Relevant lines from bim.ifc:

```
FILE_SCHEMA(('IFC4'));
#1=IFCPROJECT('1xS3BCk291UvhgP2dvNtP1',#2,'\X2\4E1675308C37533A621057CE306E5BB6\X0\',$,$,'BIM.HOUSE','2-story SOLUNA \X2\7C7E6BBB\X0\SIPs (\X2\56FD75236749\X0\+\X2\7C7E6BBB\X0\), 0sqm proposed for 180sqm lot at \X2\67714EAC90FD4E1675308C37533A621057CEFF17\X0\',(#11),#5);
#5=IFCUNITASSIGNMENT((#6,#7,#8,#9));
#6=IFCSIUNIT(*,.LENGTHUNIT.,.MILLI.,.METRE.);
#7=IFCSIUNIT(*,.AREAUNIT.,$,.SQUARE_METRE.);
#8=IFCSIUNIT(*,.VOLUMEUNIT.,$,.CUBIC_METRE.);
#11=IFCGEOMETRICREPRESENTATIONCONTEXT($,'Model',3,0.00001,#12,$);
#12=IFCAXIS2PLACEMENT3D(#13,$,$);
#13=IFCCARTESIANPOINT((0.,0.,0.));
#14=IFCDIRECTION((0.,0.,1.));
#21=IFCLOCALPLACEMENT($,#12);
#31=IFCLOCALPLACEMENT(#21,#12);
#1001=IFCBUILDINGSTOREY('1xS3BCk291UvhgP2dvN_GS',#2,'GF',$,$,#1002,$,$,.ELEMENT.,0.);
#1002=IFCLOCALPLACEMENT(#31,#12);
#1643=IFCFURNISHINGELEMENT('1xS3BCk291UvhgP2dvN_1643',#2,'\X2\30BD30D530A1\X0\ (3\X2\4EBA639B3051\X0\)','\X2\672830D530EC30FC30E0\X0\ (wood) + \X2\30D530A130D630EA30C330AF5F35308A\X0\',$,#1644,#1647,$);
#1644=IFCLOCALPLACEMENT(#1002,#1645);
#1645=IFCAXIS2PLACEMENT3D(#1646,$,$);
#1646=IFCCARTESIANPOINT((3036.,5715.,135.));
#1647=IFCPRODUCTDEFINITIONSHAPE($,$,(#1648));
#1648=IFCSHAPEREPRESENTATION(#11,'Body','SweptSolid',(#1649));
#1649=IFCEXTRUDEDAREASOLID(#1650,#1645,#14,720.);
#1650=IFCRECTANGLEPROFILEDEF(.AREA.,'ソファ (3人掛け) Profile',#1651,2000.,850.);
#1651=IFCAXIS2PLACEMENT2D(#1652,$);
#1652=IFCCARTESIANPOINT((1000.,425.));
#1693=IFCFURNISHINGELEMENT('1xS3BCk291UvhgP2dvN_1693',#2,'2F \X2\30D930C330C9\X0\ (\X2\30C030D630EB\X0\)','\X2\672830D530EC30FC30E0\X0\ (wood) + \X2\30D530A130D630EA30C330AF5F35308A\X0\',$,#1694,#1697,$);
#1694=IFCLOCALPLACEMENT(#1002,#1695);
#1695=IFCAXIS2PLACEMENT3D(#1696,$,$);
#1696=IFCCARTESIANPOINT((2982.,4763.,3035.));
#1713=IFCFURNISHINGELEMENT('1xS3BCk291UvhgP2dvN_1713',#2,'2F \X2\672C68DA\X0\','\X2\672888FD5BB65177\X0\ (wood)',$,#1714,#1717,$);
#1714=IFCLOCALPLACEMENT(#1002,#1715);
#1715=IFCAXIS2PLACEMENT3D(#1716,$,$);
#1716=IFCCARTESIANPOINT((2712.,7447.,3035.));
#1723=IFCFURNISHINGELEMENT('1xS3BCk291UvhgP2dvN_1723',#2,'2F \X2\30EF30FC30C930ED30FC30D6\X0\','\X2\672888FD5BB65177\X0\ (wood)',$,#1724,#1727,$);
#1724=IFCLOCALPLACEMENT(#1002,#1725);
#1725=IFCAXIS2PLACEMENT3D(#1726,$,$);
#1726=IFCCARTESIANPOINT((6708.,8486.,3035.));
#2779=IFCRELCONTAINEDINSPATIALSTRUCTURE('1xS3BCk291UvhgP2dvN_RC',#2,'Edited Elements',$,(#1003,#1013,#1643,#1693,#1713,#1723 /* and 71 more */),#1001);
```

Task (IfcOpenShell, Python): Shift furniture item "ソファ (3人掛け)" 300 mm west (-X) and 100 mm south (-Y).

```python
import ifcopenshell
import ifcopenshell.api.geometry
import ifcopenshell.util.placement

model = ifcopenshell.open("bim.ifc")

item = model.by_guid("1xS3BCk291UvhgP2dvN_1643")
matrix = ifcopenshell.util.placement.get_local_placement(item.ObjectPlacement)
matrix[0, 3] -= 300.0
matrix[1, 3] -= 100.0
ifcopenshell.api.geometry.edit_object_placement(model, product=item, matrix=matrix, is_si=False)

print(ifcopenshell.util.placement.get_local_placement(item.ObjectPlacement).round(3) + 0.0)

model.write("bim_edited.ifc")
```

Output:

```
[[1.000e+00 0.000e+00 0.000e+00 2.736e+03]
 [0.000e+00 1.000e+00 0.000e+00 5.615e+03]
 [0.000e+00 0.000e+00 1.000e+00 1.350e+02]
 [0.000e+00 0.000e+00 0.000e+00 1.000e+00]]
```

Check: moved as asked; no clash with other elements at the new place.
